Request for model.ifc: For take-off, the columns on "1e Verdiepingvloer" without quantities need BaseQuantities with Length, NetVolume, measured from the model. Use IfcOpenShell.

First a look at what the model holds.

```python
import ifcopenshell
import ifcopenshell.util.element
import ifcopenshell.util.unit

model = ifcopenshell.open("model.ifc")
print(model.schema)
for unit_type in ("LENGTHUNIT", "AREAUNIT", "VOLUMEUNIT"):
    print(unit_type, ifcopenshell.util.unit.calculate_unit_scale(model, unit_type))
storey = next(s for s in model.by_type("IfcBuildingStorey") if s.Name == "1e Verdiepingvloer")
columns = [e for e in ifcopenshell.util.element.get_decomposition(storey) if e.is_a("IfcColumn")]
for e in sorted(columns, key=lambda e: e.id()):
    print(e.id(), e.is_a(), e.Name, list(ifcopenshell.util.element.get_psets(e, qtos_only=True)), sep=" | ")
```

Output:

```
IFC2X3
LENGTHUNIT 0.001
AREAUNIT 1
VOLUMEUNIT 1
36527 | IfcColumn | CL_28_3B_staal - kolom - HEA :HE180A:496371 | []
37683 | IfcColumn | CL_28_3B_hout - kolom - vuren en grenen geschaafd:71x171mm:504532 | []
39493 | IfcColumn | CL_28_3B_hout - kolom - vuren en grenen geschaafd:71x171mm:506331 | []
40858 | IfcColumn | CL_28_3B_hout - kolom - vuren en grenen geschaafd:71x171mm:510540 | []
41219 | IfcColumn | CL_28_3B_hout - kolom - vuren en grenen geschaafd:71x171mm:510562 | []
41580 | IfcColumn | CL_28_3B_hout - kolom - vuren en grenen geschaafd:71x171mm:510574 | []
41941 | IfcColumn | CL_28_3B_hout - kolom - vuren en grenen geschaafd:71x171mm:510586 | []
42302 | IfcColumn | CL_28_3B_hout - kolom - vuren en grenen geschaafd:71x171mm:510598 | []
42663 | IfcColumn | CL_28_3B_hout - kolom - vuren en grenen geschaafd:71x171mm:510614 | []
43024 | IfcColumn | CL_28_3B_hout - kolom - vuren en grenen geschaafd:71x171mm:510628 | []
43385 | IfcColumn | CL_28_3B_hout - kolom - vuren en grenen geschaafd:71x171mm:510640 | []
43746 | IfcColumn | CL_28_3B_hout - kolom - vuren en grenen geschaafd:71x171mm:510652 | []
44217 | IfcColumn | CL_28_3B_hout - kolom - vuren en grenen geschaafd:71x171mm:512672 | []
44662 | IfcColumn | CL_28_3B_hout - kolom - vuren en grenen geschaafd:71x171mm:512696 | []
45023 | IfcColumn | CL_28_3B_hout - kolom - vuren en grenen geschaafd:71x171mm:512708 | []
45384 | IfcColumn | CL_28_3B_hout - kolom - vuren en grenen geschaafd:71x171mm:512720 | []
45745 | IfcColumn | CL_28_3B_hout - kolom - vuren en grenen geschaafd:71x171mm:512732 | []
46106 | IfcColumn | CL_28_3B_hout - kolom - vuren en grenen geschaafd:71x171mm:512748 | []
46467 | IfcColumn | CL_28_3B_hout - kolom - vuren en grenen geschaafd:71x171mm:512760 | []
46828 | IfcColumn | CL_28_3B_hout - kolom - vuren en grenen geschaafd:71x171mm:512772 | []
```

```python
import ifcopenshell
import ifcopenshell.api.pset
import ifcopenshell.geom
import ifcopenshell.util.element
import ifcopenshell.util.shape
import ifcopenshell.util.unit

model = ifcopenshell.open("model.ifc")
unit_scale = ifcopenshell.util.unit.calculate_unit_scale(model)
volume_scale = ifcopenshell.util.unit.calculate_unit_scale(model, "VOLUMEUNIT")
settings = ifcopenshell.geom.settings()

storey = next(s for s in model.by_type("IfcBuildingStorey") if s.Name == "1e Verdiepingvloer")
columns = [e for e in ifcopenshell.util.element.get_decomposition(storey) if e.is_a("IfcColumn")]

for e in sorted(columns, key=lambda e: e.id()):
    if ifcopenshell.util.element.get_psets(e, qtos_only=True, should_inherit=False):
        continue
    # Geometry comes back in metres, in the element's own axes.
    shape = ifcopenshell.geom.create_shape(settings, e)
    values = {
        "Length": ifcopenshell.util.shape.get_z(shape.geometry) / unit_scale,
        "NetVolume": ifcopenshell.util.shape.get_volume(shape.geometry) / volume_scale,
    }
    qto = ifcopenshell.api.pset.add_qto(model, product=e, name="BaseQuantities")
    ifcopenshell.api.pset.edit_qto(model, qto=qto, properties=values)
    print(e.id(), {k: round(v, 3) for k, v in values.items()})

model.write("model_rev.ifc")
```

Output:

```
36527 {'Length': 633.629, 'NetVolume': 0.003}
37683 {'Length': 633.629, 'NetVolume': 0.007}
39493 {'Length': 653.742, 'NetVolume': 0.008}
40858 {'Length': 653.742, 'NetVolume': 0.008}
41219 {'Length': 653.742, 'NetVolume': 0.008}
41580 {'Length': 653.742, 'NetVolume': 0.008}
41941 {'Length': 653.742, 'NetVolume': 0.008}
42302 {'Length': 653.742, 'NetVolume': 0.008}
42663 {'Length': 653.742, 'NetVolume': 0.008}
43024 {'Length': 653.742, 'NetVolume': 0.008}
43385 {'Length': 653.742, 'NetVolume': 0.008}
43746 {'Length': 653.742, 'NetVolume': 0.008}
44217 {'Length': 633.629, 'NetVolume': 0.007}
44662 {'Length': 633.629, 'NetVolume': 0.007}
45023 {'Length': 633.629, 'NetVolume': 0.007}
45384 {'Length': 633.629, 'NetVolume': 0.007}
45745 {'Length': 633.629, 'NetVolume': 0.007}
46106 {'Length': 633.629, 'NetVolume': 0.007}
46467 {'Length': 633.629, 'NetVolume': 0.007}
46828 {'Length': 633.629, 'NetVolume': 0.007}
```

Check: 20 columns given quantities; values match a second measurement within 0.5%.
